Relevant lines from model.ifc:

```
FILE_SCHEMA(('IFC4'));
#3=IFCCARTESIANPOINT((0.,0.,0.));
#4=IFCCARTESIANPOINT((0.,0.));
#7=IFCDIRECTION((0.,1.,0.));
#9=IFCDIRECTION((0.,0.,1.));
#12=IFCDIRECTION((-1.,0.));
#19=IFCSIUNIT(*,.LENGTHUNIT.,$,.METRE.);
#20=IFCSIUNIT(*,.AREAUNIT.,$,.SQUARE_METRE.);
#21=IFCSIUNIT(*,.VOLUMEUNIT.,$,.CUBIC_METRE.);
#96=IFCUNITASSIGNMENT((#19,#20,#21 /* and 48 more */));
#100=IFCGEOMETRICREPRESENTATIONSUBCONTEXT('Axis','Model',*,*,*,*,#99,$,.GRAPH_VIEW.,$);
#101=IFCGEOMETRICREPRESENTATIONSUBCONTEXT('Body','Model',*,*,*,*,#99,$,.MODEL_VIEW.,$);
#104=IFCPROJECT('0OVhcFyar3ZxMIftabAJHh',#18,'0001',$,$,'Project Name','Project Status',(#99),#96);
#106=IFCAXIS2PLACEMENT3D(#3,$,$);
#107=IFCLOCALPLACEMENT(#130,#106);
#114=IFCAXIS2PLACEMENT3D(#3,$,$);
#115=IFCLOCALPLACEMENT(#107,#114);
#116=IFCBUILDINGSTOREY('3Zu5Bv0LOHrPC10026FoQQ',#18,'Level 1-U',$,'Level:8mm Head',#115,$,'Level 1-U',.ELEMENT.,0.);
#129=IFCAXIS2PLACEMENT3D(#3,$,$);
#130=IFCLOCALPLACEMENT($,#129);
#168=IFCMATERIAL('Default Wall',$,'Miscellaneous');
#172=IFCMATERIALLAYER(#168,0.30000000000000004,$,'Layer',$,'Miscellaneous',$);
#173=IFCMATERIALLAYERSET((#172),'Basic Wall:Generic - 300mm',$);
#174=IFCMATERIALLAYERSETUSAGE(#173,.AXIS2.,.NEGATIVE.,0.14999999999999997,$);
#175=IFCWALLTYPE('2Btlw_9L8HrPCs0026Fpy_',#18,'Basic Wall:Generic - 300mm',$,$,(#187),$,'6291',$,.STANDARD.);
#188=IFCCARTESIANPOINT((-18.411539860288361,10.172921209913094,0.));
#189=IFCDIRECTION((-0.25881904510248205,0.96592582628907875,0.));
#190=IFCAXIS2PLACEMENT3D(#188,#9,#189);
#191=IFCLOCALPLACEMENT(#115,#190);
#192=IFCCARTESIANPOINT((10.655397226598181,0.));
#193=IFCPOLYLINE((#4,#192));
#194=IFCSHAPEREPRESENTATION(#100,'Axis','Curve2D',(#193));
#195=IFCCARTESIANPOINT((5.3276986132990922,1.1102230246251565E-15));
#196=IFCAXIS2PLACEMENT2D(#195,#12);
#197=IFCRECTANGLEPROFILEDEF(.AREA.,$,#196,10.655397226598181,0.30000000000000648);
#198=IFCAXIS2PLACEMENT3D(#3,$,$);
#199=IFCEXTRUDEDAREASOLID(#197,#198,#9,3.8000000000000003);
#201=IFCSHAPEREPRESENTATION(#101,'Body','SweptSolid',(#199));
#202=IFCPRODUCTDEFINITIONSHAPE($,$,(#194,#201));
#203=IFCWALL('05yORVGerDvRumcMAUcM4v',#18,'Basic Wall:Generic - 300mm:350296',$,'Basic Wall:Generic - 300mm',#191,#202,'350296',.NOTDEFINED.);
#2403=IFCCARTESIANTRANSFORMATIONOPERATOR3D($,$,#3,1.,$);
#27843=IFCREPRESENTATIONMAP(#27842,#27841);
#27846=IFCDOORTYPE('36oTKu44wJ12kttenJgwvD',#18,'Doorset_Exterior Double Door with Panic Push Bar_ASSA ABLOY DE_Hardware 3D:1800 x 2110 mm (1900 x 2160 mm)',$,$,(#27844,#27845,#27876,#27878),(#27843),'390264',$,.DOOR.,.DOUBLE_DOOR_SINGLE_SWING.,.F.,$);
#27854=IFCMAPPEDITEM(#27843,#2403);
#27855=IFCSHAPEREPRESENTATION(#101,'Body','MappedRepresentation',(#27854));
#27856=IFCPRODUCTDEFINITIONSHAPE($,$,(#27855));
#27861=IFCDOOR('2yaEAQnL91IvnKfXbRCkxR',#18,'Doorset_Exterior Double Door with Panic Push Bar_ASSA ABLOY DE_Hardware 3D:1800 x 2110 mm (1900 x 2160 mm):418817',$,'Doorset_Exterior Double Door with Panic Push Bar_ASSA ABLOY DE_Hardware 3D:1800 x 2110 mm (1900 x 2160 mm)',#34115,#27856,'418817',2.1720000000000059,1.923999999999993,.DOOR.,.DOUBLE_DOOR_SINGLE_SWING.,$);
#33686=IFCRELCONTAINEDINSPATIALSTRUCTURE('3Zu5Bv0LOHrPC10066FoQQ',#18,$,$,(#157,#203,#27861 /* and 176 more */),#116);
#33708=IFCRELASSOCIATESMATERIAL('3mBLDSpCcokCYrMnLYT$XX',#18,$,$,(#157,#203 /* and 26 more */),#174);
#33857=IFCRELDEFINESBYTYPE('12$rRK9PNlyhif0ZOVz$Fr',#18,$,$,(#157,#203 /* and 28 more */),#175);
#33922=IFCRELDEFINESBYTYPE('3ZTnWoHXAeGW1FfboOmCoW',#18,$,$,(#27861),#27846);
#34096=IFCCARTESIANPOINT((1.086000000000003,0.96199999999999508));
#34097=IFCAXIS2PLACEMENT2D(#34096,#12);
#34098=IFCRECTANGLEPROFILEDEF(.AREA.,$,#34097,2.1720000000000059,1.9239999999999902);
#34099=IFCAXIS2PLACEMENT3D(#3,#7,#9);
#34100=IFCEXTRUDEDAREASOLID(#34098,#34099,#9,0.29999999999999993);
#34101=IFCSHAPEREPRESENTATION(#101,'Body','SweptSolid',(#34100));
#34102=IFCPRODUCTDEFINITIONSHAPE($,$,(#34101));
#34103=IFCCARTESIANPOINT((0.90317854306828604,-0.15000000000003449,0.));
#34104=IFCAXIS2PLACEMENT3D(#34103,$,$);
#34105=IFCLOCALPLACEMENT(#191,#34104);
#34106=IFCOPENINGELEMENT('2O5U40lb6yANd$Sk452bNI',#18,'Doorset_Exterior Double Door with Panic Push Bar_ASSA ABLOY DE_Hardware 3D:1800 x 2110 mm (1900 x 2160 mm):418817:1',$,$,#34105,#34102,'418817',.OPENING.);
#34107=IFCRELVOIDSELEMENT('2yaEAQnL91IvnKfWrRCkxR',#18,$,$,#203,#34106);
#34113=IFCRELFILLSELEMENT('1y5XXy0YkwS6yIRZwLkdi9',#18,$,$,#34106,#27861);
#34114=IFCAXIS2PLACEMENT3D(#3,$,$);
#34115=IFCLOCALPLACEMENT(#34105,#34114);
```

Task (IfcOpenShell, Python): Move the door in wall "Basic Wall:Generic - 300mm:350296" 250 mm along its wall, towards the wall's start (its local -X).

```python
import ifcopenshell
import ifcopenshell.api.geometry
import ifcopenshell.util.placement
import ifcopenshell.util.unit

model = ifcopenshell.open("model.ifc")
unit_scale = ifcopenshell.util.unit.calculate_unit_scale(model)

door = model.by_id(27861)
opening = door.FillsVoids[0].RelatingOpeningElement
wall = opening.VoidsElements[0].RelatingBuildingElement

wall_matrix = ifcopenshell.util.placement.get_local_placement(wall.ObjectPlacement)
shift = wall_matrix[:3, 0] * -0.25 / unit_scale
before = ifcopenshell.util.placement.get_local_placement(door.ObjectPlacement)[:3, 3].copy()

# The door is placed relative to its opening, so it follows when the opening moves.
matrix = ifcopenshell.util.placement.get_local_placement(opening.ObjectPlacement)
matrix[:3, 3] += shift
ifcopenshell.api.geometry.edit_object_placement(
    model, product=opening, matrix=matrix, is_si=False, should_transform_children=True
)

after = ifcopenshell.util.placement.get_local_placement(door.ObjectPlacement)[:3, 3]
print("door moved by", (after - before).round(3) + 0.0)

model.write("model_edited.ifc")
```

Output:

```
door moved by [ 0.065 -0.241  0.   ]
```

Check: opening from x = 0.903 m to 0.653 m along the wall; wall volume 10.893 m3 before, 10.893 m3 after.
